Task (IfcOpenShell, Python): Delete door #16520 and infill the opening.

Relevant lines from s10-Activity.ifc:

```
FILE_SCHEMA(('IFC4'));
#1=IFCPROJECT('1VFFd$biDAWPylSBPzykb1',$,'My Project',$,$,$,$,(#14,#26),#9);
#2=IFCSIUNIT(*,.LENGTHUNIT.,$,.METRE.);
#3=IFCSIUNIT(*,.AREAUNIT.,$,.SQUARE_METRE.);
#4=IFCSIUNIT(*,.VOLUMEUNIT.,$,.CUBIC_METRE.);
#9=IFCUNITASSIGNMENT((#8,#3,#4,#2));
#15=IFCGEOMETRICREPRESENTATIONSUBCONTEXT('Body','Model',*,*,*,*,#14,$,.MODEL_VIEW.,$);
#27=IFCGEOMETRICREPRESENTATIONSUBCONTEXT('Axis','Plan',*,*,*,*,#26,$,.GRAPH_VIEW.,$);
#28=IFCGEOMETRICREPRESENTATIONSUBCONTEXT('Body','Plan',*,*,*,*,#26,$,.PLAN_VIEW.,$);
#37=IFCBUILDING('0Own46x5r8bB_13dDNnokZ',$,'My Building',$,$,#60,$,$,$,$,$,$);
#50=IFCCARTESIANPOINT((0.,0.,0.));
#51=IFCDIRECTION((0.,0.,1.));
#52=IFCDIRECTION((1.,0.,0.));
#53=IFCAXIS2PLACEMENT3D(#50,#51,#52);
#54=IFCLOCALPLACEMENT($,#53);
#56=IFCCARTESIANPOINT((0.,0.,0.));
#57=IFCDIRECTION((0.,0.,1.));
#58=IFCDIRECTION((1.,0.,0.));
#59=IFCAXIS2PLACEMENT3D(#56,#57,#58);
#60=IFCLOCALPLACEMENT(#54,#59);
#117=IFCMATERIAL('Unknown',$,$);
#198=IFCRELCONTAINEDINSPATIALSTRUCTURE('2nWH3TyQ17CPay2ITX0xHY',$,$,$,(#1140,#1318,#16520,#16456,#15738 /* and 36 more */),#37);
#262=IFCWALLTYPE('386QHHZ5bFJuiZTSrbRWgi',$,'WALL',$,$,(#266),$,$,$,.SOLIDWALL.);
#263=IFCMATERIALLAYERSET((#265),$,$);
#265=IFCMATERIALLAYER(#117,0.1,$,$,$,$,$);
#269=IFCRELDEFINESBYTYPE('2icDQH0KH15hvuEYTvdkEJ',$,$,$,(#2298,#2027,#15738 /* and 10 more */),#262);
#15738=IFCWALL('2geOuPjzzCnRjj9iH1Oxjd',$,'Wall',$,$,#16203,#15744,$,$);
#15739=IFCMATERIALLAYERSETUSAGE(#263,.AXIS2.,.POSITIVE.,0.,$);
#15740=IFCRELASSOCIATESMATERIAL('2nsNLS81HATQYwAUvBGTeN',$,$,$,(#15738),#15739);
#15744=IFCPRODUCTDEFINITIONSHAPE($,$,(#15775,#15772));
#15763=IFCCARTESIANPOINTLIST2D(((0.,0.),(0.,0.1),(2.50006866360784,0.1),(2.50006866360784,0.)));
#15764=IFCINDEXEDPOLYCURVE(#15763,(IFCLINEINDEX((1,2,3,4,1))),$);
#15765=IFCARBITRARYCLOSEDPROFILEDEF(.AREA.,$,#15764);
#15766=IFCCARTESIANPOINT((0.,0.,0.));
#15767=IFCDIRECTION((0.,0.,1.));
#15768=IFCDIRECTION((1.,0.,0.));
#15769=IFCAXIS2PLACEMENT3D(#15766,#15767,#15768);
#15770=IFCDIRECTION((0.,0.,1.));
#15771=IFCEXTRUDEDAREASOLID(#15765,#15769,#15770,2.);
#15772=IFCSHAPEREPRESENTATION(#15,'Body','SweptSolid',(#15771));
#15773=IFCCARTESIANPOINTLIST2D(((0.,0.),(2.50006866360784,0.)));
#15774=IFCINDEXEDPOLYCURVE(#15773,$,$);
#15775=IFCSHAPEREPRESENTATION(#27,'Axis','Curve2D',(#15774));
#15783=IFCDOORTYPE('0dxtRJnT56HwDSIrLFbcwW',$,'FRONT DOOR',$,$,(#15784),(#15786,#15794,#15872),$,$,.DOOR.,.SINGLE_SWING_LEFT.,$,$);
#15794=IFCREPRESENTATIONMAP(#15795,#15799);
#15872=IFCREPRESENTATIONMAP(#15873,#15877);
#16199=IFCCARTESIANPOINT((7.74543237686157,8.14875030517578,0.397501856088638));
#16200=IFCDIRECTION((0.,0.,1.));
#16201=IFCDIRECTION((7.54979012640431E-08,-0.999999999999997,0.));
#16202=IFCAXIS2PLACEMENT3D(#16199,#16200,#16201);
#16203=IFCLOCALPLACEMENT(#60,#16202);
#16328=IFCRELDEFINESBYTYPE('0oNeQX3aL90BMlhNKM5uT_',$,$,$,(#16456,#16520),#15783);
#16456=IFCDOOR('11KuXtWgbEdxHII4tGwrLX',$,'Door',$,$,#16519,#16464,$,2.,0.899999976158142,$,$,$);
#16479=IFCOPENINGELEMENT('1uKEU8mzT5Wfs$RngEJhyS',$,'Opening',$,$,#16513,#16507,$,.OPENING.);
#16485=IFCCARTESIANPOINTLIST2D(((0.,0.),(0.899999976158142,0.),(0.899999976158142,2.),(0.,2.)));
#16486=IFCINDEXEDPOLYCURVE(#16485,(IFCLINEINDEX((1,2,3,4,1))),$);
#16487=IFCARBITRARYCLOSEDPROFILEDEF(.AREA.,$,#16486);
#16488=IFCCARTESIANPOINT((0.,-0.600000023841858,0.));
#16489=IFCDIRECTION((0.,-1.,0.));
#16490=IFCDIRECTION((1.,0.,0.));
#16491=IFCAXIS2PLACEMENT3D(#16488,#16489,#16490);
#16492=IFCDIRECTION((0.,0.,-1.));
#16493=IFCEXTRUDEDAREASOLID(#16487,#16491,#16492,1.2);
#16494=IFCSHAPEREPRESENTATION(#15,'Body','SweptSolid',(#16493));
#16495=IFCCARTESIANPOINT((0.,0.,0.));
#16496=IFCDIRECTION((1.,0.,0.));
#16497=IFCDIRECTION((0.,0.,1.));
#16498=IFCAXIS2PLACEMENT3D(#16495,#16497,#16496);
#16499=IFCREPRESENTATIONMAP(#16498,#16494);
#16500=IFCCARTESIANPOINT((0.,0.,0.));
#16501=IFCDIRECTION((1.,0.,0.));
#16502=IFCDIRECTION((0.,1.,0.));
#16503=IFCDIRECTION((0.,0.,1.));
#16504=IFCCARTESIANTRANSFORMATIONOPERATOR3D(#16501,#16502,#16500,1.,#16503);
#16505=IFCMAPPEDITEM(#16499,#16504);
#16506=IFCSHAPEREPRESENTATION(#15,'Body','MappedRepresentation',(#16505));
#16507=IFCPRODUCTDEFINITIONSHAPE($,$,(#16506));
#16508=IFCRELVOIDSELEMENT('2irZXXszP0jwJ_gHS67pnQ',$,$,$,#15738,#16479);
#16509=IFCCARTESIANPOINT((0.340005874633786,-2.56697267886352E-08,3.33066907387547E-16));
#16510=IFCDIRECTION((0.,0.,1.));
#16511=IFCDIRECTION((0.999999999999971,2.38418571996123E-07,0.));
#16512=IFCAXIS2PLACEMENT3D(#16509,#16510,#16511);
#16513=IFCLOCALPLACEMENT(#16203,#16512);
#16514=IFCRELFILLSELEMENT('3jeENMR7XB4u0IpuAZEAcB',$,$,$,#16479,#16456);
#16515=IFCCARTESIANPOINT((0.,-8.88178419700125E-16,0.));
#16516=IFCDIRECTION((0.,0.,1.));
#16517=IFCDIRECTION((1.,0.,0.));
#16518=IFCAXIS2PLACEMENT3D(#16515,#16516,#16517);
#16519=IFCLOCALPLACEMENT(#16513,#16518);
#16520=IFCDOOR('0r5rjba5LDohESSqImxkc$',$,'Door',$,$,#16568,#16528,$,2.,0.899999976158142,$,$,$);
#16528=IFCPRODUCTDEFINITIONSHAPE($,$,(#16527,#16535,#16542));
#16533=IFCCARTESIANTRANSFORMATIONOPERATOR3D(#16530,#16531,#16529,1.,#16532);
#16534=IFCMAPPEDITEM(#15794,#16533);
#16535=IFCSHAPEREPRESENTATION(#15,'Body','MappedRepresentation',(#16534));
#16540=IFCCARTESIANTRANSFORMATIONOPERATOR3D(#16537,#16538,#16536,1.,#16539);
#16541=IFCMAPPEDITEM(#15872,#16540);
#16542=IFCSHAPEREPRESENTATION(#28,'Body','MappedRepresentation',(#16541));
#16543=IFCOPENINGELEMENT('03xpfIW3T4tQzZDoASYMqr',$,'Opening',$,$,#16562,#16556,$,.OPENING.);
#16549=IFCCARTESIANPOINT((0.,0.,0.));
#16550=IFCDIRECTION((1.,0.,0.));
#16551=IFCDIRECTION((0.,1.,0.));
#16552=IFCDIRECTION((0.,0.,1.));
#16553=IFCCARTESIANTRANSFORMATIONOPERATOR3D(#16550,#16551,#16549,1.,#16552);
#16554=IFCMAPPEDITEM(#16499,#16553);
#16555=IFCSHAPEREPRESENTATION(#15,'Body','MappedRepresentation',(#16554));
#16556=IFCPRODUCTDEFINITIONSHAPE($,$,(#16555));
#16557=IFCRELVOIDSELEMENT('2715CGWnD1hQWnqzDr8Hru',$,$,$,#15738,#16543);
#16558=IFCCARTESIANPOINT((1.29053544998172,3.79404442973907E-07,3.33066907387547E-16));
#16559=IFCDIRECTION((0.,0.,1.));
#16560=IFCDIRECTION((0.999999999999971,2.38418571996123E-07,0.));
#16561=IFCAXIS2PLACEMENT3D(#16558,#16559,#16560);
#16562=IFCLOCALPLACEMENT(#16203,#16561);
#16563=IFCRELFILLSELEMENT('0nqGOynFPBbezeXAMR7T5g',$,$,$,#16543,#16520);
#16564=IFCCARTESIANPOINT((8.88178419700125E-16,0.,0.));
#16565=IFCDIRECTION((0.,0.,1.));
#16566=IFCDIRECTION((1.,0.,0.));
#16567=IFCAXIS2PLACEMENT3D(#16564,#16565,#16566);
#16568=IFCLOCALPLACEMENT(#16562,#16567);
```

```python
import ifcopenshell
import ifcopenshell.api.feature
import ifcopenshell.api.root
import ifcopenshell.geom
import ifcopenshell.util.shape

model = ifcopenshell.open("s10-Activity.ifc")
settings = ifcopenshell.geom.settings()


def volume(element):
    """Net volume in cubic metres, openings subtracted."""
    shape = ifcopenshell.geom.create_shape(settings, element)
    return ifcopenshell.util.shape.get_volume(shape.geometry)


door = model.by_guid("0r5rjba5LDohESSqImxkc$")
opening = door.FillsVoids[0].RelatingOpeningElement
wall = opening.VoidsElements[0].RelatingBuildingElement
before = volume(wall)

ifcopenshell.api.root.remove_product(model, product=door)
ifcopenshell.api.feature.remove_feature(model, feature=opening)

after = volume(wall)

print(f"wall volume {before:.3f} -> {after:.3f} m3")

model.write("s10-Activity_edited.ifc")
```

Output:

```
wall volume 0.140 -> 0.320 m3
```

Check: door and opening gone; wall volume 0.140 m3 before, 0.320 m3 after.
